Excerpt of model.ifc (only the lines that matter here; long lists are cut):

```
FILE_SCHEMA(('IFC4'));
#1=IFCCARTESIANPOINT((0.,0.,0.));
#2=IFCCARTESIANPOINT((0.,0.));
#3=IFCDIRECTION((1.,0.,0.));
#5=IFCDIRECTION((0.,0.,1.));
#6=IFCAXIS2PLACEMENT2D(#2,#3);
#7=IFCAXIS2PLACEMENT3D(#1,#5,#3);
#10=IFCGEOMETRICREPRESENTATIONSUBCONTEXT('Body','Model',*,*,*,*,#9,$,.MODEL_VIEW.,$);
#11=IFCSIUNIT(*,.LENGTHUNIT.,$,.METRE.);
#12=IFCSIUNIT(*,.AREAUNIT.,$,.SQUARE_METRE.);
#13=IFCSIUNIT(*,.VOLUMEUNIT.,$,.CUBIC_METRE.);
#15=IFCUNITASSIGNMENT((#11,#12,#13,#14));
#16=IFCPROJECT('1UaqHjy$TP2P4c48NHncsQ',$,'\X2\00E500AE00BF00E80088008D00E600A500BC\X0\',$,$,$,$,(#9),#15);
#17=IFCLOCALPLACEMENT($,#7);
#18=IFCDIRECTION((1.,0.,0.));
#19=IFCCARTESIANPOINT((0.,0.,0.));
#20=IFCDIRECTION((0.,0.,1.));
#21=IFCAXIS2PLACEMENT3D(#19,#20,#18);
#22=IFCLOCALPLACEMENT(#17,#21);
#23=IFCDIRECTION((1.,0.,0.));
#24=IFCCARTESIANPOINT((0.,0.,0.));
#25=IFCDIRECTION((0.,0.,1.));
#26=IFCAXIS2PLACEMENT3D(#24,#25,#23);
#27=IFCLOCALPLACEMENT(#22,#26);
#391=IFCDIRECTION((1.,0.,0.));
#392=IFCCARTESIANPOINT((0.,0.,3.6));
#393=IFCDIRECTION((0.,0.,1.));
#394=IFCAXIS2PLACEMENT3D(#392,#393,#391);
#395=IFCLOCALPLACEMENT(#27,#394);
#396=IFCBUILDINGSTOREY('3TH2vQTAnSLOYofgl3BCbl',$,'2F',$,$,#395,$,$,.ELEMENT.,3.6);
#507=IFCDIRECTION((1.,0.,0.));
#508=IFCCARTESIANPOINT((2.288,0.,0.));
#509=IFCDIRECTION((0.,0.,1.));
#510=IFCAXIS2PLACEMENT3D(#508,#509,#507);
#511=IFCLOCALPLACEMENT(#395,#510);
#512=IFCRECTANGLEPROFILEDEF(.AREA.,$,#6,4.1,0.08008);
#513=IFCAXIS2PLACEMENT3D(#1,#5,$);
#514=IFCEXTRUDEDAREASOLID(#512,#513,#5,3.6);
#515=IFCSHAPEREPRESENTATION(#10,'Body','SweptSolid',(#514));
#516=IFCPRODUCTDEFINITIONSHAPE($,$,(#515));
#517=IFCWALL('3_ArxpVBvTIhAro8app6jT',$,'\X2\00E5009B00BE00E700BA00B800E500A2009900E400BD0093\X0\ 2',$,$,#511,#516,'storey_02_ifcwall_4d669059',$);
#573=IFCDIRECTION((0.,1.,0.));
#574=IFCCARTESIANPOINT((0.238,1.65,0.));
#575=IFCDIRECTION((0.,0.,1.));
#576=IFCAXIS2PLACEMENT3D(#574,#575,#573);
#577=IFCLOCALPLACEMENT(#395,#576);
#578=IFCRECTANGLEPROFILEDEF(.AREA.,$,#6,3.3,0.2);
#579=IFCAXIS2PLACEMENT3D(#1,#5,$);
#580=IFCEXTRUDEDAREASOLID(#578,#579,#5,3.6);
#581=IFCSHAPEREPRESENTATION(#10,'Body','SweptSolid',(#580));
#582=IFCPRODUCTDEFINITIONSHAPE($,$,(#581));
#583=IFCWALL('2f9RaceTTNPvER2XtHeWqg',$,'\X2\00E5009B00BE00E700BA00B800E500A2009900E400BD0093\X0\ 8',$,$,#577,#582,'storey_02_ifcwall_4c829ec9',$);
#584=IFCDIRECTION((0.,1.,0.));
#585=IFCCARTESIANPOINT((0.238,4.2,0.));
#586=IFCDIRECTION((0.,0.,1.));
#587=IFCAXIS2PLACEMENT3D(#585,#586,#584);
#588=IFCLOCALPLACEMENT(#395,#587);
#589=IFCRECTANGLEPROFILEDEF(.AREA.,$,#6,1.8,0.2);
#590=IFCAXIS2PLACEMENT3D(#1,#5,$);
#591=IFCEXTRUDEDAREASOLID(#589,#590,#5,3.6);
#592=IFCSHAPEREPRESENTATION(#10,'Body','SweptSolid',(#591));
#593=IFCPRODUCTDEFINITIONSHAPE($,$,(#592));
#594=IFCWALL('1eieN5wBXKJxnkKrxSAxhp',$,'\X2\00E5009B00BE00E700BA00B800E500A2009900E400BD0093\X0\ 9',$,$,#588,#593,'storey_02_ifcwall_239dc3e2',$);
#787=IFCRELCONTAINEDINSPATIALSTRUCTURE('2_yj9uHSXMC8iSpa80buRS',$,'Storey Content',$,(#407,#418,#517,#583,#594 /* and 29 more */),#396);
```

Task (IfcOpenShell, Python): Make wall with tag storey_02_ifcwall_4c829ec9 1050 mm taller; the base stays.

```python
import ifcopenshell
import ifcopenshell.geom
import ifcopenshell.util.representation
import ifcopenshell.util.shape
import ifcopenshell.util.unit

model = ifcopenshell.open("model.ifc")
unit_scale = ifcopenshell.util.unit.calculate_unit_scale(model)
settings = ifcopenshell.geom.settings()


def volume(element):
    """Net volume in cubic metres, openings subtracted."""
    shape = ifcopenshell.geom.create_shape(settings, element)
    return ifcopenshell.util.shape.get_volume(shape.geometry)


wall = model.by_guid("2f9RaceTTNPvER2XtHeWqg")
before = volume(wall)

body = ifcopenshell.util.representation.get_representation(wall, "Model", "Body")
solid = body.Items[0]
old_height = solid.Depth
solid.Depth += 1.05 / unit_scale
after = volume(wall)

print(f"height {old_height:g} -> {solid.Depth:g}, volume {before:.3f} -> {after:.3f} m3")

model.write("model-out.ifc")
```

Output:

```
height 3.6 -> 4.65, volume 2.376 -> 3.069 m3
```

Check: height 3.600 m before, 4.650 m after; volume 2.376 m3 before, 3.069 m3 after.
